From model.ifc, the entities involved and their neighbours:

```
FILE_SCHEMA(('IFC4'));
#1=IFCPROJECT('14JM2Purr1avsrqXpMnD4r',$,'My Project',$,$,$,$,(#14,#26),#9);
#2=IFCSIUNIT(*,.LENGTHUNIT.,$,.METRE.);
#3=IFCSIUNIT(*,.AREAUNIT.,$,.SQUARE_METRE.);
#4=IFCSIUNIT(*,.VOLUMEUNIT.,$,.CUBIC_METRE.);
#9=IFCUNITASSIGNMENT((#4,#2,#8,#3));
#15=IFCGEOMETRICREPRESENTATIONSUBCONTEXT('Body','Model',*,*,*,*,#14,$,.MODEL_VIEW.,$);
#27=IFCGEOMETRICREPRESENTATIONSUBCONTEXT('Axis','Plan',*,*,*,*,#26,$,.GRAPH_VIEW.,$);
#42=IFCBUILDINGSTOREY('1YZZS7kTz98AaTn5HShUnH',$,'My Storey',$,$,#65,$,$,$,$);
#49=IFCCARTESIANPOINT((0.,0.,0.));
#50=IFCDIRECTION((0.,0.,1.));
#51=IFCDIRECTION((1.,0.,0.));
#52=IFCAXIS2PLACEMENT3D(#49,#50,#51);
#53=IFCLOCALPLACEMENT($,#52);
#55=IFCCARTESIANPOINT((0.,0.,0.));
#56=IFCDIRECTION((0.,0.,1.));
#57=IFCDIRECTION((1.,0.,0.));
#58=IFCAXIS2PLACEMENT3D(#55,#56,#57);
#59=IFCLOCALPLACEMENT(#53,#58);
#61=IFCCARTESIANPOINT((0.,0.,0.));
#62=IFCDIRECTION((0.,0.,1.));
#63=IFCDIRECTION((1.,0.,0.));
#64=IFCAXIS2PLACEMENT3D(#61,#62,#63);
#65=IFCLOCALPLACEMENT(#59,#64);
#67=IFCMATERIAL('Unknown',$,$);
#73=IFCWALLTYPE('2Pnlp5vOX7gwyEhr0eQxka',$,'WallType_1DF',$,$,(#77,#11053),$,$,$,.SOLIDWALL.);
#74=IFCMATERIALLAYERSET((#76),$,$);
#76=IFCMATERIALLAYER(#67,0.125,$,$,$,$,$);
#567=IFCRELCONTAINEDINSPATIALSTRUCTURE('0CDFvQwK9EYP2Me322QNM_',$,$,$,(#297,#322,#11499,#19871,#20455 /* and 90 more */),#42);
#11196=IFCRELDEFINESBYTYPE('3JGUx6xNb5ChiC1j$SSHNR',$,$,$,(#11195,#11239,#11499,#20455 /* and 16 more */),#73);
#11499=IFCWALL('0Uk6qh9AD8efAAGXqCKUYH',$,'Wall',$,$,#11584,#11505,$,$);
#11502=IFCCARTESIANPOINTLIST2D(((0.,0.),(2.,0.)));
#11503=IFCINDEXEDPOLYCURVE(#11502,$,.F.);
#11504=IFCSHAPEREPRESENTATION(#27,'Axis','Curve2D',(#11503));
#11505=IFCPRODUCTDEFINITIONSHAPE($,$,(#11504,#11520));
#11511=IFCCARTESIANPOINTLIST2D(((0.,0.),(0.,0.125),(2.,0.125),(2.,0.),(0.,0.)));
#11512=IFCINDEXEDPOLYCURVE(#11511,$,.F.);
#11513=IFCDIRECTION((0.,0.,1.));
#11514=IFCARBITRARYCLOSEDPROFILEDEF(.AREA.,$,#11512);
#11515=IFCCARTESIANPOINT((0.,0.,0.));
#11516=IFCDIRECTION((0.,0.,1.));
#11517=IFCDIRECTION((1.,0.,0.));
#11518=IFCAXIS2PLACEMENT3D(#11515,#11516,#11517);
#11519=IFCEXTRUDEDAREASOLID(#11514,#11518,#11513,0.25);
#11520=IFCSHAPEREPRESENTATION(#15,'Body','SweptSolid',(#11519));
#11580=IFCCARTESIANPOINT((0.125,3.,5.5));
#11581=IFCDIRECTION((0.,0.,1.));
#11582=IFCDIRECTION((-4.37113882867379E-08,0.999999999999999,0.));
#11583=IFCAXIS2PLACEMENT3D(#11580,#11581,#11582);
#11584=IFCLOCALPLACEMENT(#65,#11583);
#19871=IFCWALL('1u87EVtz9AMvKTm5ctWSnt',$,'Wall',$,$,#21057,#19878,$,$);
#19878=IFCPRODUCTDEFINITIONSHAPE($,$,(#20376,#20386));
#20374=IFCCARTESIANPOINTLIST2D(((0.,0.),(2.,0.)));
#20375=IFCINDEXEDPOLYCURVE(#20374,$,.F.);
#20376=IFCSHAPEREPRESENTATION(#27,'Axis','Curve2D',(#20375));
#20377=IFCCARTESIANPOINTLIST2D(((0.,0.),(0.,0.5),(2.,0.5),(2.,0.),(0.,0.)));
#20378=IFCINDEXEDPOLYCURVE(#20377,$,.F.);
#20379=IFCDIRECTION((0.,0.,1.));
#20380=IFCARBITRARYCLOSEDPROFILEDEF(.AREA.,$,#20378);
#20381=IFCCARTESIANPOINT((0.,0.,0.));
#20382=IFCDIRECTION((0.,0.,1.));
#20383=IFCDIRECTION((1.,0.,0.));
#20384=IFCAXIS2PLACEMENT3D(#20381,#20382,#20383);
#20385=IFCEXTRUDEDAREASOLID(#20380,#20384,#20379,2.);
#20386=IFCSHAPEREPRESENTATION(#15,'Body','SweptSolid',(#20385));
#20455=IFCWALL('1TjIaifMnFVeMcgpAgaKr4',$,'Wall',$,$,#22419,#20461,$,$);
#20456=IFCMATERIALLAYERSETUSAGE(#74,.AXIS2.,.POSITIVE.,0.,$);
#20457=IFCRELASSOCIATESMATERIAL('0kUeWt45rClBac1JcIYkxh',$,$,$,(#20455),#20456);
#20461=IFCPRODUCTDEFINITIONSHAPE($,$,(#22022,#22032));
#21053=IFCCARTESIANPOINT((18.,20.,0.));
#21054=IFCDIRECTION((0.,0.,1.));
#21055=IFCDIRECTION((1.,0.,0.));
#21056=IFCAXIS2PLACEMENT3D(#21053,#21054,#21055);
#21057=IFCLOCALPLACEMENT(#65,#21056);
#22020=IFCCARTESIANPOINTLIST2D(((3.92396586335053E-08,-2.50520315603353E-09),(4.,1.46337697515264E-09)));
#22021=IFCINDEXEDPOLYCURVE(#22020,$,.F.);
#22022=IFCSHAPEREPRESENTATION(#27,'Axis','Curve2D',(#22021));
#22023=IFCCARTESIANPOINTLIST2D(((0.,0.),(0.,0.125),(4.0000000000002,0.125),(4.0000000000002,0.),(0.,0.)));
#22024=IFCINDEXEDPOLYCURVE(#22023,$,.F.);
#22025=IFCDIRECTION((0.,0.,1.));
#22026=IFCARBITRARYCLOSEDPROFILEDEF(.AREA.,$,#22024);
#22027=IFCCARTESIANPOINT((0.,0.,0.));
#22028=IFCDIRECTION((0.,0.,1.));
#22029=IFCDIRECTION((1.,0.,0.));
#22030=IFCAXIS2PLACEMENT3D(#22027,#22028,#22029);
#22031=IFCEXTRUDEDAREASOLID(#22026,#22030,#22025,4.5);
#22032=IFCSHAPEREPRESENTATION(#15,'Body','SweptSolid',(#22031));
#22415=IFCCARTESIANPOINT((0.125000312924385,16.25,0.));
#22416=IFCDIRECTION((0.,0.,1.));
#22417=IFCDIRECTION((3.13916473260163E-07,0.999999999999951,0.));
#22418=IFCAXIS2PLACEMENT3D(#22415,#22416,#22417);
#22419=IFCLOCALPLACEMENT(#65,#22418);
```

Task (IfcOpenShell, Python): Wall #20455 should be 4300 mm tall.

```python
import ifcopenshell
import ifcopenshell.geom
import ifcopenshell.util.representation
import ifcopenshell.util.shape
import ifcopenshell.util.unit

model = ifcopenshell.open("model.ifc")
unit_scale = ifcopenshell.util.unit.calculate_unit_scale(model)
settings = ifcopenshell.geom.settings()


def volume(element):
    """Net volume in cubic metres, openings subtracted."""
    shape = ifcopenshell.geom.create_shape(settings, element)
    return ifcopenshell.util.shape.get_volume(shape.geometry)


wall = model.by_guid("1TjIaifMnFVeMcgpAgaKr4")
before = volume(wall)

body = ifcopenshell.util.representation.get_representation(wall, "Model", "Body")
solid = body.Items[0]
old_height = solid.Depth
solid.Depth = 4.3 / unit_scale
after = volume(wall)

print(f"height {old_height:g} -> {solid.Depth:g}, volume {before:.3f} -> {after:.3f} m3")

model.write("model_v2.ifc")
```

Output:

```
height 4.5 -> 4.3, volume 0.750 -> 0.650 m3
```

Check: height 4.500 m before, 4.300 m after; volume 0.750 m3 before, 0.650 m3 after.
